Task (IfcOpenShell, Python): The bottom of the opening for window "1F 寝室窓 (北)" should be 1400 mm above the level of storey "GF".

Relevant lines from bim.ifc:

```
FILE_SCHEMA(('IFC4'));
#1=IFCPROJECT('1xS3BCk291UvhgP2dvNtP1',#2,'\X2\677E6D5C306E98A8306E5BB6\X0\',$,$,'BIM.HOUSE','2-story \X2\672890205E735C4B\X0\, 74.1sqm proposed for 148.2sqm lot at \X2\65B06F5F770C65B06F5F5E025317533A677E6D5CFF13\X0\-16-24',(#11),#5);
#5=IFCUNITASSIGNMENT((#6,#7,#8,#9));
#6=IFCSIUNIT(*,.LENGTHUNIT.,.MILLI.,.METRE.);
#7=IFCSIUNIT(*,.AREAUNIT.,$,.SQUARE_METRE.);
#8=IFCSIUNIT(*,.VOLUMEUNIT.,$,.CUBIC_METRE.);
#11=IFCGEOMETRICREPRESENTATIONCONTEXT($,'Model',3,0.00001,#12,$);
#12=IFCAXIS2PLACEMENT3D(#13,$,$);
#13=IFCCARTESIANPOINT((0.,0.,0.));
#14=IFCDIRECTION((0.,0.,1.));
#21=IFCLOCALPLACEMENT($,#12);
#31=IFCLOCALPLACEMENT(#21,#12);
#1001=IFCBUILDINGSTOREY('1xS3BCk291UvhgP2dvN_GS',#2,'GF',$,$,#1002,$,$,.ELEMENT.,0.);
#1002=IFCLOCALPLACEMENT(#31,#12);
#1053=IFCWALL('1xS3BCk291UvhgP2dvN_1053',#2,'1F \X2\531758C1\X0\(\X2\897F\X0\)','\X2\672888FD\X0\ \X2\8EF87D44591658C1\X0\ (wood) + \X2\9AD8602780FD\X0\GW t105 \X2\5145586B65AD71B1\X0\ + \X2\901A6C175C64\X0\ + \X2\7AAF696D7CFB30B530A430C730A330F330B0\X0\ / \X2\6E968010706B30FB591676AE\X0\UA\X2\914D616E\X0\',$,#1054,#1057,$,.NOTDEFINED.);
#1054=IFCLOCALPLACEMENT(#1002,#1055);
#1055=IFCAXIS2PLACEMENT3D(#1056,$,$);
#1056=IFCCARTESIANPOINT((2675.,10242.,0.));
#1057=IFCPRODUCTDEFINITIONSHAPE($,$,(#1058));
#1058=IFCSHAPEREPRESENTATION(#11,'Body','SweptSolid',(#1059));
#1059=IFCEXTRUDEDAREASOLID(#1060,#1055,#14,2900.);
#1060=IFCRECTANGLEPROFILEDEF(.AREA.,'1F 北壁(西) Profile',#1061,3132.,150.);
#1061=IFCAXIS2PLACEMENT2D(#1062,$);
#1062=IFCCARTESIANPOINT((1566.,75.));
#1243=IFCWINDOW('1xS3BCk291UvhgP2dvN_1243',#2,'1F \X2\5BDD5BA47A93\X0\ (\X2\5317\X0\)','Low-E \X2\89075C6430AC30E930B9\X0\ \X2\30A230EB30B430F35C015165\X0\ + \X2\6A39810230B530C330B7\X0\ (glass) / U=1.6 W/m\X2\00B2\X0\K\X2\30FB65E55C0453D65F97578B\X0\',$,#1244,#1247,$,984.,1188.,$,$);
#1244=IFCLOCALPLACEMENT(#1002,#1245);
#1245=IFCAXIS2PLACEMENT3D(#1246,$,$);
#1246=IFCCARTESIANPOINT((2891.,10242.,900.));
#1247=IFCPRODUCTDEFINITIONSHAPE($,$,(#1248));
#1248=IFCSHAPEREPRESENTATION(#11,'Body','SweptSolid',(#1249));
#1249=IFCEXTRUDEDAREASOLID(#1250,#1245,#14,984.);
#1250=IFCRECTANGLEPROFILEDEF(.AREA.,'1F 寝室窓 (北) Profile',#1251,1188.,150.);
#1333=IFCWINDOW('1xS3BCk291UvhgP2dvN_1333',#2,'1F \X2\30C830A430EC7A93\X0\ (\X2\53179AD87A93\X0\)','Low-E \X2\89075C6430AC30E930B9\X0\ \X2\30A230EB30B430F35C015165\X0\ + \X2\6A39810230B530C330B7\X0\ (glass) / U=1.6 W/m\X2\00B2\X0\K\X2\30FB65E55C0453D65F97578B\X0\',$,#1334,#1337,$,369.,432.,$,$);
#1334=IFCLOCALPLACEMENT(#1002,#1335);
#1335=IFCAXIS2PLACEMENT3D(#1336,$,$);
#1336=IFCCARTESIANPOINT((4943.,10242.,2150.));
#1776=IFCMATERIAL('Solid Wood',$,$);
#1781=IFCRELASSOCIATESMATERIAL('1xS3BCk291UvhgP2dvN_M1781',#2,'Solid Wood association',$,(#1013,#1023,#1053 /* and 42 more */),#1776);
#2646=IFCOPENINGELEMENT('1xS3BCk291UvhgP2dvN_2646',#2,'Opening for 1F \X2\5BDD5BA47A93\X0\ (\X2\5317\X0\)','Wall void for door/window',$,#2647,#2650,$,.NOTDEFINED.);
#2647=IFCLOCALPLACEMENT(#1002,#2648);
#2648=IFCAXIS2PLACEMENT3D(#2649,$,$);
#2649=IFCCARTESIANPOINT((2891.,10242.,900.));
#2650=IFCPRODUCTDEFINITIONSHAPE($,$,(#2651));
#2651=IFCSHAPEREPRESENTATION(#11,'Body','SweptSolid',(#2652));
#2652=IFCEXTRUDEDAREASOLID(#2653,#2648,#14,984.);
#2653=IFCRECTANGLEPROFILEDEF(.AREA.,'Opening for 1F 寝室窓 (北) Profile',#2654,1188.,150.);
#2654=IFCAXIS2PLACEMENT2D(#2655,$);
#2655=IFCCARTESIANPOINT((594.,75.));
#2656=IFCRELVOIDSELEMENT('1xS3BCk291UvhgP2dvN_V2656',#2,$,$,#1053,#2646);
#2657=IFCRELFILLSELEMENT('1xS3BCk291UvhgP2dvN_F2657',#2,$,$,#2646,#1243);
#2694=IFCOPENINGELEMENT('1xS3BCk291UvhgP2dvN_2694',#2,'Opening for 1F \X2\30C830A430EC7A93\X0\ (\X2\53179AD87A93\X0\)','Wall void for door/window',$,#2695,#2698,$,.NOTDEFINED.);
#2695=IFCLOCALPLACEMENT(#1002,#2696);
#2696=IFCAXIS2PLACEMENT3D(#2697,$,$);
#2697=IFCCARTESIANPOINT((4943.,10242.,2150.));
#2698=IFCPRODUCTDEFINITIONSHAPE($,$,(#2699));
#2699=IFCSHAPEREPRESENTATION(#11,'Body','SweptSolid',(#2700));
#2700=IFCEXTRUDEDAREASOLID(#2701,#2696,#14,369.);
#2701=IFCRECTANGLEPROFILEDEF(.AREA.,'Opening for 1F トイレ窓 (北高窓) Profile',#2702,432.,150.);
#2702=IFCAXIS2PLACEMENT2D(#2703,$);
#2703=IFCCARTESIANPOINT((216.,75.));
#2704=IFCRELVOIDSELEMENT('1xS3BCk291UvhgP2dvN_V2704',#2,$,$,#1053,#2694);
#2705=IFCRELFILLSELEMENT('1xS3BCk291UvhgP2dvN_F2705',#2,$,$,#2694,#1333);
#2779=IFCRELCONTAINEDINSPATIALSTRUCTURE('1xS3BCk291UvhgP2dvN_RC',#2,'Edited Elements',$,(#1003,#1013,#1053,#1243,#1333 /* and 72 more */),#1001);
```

```python
import numpy as np
import ifcopenshell
import ifcopenshell.api.geometry
import ifcopenshell.geom
import ifcopenshell.util.element
import ifcopenshell.util.placement
import ifcopenshell.util.shape
import ifcopenshell.util.unit

model = ifcopenshell.open("bim.ifc")
unit_scale = ifcopenshell.util.unit.calculate_unit_scale(model)

window = model.by_guid("1xS3BCk291UvhgP2dvN_1243")
opening = window.FillsVoids[0].RelatingOpeningElement
storey = ifcopenshell.util.element.get_container(window, ifc_class="IfcBuildingStorey")
level = ifcopenshell.util.placement.get_local_placement(storey.ObjectPlacement)[2, 3]

# The opening's origin need not be at the sill, so measure its lowest point.
shape = ifcopenshell.geom.create_shape(ifcopenshell.geom.settings(), opening)
bottom = ifcopenshell.util.shape.get_shape_bottom_elevation(shape, shape.geometry) / unit_scale
dz = level + 1.4 / unit_scale - bottom

shift = np.array([0.0, 0.0, dz])
# The window is not placed relative to its opening, so move both.
for product in (opening, window):
    matrix = ifcopenshell.util.placement.get_local_placement(product.ObjectPlacement)
    matrix[:3, 3] += shift
    ifcopenshell.api.geometry.edit_object_placement(model, product=product, matrix=matrix, is_si=False)

print(f"moved by {dz * unit_scale:+.3f} m")

model.write("bim-out.ifc")
```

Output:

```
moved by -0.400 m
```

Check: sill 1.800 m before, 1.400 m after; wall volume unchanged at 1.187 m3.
